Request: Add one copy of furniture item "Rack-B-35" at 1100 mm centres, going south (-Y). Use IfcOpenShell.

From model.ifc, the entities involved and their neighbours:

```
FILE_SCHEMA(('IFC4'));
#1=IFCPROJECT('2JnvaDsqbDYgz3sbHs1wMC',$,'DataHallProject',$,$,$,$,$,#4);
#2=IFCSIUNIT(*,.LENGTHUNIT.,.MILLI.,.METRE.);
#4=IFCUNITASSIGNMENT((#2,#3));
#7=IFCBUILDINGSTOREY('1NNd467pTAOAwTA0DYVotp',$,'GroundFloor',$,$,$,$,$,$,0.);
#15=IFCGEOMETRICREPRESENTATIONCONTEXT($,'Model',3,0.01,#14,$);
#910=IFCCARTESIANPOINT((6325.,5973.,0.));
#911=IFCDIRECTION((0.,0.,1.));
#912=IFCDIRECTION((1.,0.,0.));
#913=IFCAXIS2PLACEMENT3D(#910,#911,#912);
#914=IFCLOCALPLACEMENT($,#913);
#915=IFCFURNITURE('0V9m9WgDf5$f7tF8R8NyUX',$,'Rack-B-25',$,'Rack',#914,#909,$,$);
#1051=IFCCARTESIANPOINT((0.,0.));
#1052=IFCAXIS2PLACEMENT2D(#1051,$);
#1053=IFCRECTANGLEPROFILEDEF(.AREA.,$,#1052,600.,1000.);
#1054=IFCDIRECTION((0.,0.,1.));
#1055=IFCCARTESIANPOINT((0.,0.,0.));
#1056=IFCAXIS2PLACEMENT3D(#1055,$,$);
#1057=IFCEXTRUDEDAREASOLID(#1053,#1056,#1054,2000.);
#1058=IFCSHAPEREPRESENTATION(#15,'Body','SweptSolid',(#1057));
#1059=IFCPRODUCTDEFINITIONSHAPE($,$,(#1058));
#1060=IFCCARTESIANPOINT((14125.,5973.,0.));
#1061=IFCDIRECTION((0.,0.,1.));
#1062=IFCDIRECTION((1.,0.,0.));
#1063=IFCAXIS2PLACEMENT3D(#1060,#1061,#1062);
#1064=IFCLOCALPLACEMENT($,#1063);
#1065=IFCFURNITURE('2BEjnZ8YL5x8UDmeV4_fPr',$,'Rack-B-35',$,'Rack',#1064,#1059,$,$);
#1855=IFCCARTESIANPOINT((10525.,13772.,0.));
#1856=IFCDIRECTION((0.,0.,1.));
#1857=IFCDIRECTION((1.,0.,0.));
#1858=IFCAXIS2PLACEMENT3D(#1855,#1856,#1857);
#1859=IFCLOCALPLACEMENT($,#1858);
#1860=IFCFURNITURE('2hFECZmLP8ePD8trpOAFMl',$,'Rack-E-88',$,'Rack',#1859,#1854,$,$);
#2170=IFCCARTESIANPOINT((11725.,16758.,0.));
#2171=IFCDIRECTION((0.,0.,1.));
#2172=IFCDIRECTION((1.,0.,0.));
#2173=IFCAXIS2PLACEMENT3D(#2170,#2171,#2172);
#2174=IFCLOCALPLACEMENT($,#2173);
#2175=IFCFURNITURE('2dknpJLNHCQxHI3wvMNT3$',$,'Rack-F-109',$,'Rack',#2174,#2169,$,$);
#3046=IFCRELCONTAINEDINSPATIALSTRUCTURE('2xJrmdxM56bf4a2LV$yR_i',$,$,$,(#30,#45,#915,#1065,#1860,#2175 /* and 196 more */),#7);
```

```python
import numpy as np
import ifcopenshell
import ifcopenshell.api.geometry
import ifcopenshell.api.root
import ifcopenshell.util.element
import ifcopenshell.util.placement
import ifcopenshell.util.unit

model = ifcopenshell.open("model.ifc")
unit_scale = ifcopenshell.util.unit.calculate_unit_scale(model)

source = model.by_guid("2BEjnZ8YL5x8UDmeV4_fPr")
base = ifcopenshell.util.placement.get_local_placement(source.ObjectPlacement)
step = np.array([0.0, -1.0, 0.0]) * 1.1 / unit_scale

for i in range(1, 2):
    copy = ifcopenshell.api.root.copy_class(model, product=source)
    copy.Representation = ifcopenshell.util.element.copy_deep(
        model, source.Representation, exclude=["IfcGeometricRepresentationContext", "IfcRepresentationMap"]
    )
    matrix = base.copy()
    matrix[:3, 3] += i * step
    print("added at", matrix[:3, 3].round(3) + 0.0)
    ifcopenshell.api.geometry.edit_object_placement(model, product=copy, matrix=matrix, is_si=False)

model.write("model_v2.ifc")
```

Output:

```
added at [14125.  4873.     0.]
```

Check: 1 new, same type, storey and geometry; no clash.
